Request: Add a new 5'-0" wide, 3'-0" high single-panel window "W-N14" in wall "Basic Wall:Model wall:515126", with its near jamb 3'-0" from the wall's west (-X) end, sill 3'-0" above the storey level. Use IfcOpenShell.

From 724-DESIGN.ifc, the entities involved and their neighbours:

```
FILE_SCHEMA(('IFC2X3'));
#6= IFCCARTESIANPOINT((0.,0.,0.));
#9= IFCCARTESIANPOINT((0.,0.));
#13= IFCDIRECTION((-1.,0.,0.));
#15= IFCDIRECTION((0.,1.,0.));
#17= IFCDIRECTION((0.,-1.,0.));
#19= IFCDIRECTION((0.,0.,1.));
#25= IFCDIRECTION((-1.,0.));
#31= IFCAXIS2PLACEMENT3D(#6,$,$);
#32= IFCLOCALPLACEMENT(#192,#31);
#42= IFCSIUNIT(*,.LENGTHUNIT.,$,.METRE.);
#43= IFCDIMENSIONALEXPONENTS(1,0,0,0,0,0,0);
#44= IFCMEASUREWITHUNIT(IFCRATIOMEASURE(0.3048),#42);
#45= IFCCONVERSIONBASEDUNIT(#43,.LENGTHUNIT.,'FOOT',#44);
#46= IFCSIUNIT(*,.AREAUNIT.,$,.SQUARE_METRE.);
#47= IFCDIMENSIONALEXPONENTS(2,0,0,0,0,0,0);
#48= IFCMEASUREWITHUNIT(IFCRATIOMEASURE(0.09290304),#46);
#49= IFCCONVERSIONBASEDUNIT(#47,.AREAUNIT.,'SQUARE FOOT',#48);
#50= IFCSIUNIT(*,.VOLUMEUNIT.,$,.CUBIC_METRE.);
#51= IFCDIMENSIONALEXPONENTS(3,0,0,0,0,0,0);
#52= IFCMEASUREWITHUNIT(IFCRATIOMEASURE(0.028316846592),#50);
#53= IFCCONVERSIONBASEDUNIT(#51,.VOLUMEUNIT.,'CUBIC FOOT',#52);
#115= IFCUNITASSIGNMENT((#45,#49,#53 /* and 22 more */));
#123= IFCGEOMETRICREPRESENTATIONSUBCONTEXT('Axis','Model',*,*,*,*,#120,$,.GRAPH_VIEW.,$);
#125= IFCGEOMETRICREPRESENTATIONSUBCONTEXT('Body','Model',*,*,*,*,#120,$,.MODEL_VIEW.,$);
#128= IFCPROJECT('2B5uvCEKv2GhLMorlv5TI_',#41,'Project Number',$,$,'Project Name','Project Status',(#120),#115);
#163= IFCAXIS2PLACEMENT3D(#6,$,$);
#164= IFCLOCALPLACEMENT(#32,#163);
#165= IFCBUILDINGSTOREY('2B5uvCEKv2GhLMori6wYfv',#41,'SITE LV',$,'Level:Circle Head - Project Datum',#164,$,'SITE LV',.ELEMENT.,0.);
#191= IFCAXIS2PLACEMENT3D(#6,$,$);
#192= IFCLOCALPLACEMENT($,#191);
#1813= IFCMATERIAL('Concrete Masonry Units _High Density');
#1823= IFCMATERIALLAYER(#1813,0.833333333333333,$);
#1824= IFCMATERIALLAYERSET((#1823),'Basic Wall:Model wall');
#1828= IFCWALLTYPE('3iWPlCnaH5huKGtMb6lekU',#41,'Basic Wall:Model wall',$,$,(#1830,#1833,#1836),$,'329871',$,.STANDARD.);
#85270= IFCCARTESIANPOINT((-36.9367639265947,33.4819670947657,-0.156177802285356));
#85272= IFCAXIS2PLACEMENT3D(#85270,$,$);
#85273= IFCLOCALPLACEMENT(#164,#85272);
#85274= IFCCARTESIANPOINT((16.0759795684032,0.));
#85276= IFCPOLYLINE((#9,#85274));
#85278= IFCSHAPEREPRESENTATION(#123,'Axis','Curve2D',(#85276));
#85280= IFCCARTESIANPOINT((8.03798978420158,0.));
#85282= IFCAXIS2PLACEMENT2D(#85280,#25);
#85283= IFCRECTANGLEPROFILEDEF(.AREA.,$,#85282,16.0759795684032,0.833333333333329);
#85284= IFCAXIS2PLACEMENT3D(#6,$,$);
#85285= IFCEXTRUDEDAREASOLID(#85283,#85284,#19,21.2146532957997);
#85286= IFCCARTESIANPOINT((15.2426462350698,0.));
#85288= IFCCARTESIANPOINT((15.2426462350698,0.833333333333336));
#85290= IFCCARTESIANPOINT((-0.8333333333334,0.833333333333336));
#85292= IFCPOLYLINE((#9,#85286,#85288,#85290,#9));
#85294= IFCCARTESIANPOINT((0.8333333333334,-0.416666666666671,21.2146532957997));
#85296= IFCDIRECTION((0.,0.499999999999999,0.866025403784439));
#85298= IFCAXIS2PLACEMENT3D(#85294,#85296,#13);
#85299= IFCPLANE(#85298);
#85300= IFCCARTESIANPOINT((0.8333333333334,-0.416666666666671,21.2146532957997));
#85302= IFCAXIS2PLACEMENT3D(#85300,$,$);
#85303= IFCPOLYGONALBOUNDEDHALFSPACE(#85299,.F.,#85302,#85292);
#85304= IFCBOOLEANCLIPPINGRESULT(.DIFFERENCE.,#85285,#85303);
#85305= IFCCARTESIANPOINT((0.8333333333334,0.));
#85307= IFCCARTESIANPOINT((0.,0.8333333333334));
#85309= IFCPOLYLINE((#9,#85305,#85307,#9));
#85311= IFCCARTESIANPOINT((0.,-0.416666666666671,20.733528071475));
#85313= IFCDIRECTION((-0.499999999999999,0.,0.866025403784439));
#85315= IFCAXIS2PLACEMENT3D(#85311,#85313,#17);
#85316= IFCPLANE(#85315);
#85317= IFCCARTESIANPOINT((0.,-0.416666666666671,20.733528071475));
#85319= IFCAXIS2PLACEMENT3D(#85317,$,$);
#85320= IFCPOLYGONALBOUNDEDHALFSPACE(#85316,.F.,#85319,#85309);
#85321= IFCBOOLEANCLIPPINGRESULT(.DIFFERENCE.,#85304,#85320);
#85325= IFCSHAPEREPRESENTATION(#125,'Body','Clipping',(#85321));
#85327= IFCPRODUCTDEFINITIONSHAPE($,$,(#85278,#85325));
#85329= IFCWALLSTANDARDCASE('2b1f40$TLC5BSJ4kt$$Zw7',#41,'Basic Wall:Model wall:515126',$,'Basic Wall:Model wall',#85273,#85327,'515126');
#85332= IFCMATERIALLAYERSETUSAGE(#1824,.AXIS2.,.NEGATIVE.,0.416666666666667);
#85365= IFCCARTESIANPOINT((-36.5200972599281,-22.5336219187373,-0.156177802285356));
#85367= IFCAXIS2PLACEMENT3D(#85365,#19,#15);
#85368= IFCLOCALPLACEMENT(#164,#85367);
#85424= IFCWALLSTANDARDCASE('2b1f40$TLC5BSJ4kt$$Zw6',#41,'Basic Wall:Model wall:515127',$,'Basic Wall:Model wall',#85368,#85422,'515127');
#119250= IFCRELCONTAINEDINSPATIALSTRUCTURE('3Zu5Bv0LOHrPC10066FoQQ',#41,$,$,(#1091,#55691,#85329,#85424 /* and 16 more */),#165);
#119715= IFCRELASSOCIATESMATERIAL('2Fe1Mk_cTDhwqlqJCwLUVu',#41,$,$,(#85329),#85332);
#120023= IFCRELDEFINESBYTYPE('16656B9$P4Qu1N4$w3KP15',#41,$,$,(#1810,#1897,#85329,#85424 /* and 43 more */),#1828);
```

```python
import numpy as np
import ifcopenshell
import ifcopenshell.api.feature
import ifcopenshell.api.geometry
import ifcopenshell.api.root
import ifcopenshell.api.spatial
import ifcopenshell.api.type
import ifcopenshell.geom
import ifcopenshell.util.element
import ifcopenshell.util.placement
import ifcopenshell.util.representation
import ifcopenshell.util.shape
import ifcopenshell.util.unit

model = ifcopenshell.open("724-DESIGN.ifc")
unit_scale = ifcopenshell.util.unit.calculate_unit_scale(model)
settings = ifcopenshell.geom.settings()


def volume(element):
    """Net volume in cubic metres, openings subtracted."""
    shape = ifcopenshell.geom.create_shape(settings, element)
    return ifcopenshell.util.shape.get_volume(shape.geometry)


wall = model.by_guid("2b1f40$TLC5BSJ4kt$$Zw7")
storey = ifcopenshell.util.element.get_container(wall, ifc_class="IfcBuildingStorey")
context = ifcopenshell.util.representation.get_context(model, "Model", "Body", "MODEL_VIEW")
before = volume(wall)

width, height, from_end, sill = 1.524, 0.9144, 0.9144, 0.9144  # metres

# The wall runs along its own X axis, and the end named is its -X end.
wall_shape = ifcopenshell.geom.create_shape(settings, wall)
x, y, z = ifcopenshell.util.shape.get_vertices(wall_shape.geometry).T
start = x.min() + from_end
face, thickness = float(y.min()), float(y.max() - y.min())
wall_matrix = ifcopenshell.util.placement.get_local_placement(wall.ObjectPlacement)
level = ifcopenshell.util.placement.get_local_placement(storey.ObjectPlacement)[2, 3]


def in_wall(x, y):
    """Placement at x, y metres in the wall's axes, at sill height."""
    matrix = wall_matrix.copy()
    matrix[:, 3] = wall_matrix @ np.array([x / unit_scale, y / unit_scale, 0.0, 1.0])
    matrix[2, 3] = level + sill / unit_scale
    return matrix


# Opening: a box that overshoots both wall faces by 50 mm.
opening = ifcopenshell.api.root.create_entity(model, ifc_class="IfcOpeningElement")
box = ifcopenshell.api.geometry.add_wall_representation(
    model, context=context, length=width, height=height, thickness=thickness + 0.1
)
ifcopenshell.api.geometry.assign_representation(model, product=opening, representation=box)
ifcopenshell.api.geometry.edit_object_placement(model, product=opening, matrix=in_wall(start, face - 0.05), is_si=False)
ifcopenshell.api.feature.add_feature(model, feature=opening, element=wall)

window = ifcopenshell.api.root.create_entity(model, ifc_class="IfcWindow", name="W-N14")
window.OverallWidth, window.OverallHeight = width / unit_scale, height / unit_scale
body = ifcopenshell.api.geometry.add_window_representation(
    model,
    context=context,
    overall_width=window.OverallWidth,
    overall_height=window.OverallHeight,
    partition_type="SINGLE_PANEL",
)
ifcopenshell.api.geometry.assign_representation(model, product=window, representation=body)
ifcopenshell.api.spatial.assign_container(model, products=[window], relating_structure=storey)
fills = ifcopenshell.api.feature.add_filling(model, opening=opening, element=window)
fills.OwnerHistory = window.OwnerHistory  # required in IFC2X3

# IFC2X3 keeps the operation on the window style.
style = ifcopenshell.api.root.create_entity(model, ifc_class="IfcWindowStyle", name="W-N14")
style.OperationType, style.ConstructionType = "SINGLE_PANEL", "NOTDEFINED"
style.ParameterTakesPrecedence = style.Sizeable = False
ifcopenshell.api.type.assign_type(model, related_objects=[window], relating_type=style)

# Centre the window in the wall's thickness.
ifcopenshell.api.geometry.edit_object_placement(model, product=window, matrix=in_wall(start, face), is_si=False)
window_shape = ifcopenshell.geom.create_shape(settings, window)
depth = ifcopenshell.util.shape.get_vertices(window_shape.geometry)[:, 1]
offset = face + thickness / 2 - (depth.min() + depth.max()) / 2
ifcopenshell.api.geometry.edit_object_placement(model, product=window, matrix=in_wall(start, offset), is_si=False)

after = volume(wall)

print(f"wall volume {before:.3f} -> {after:.3f} m3")

model.write("724-DESIGN_v2.ifc")
```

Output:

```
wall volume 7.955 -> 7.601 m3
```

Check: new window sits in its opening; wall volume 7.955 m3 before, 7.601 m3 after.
